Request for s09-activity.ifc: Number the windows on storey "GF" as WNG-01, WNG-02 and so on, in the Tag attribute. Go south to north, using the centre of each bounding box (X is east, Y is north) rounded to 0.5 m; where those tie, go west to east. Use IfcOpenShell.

First a look at what the model holds.

```python
import ifcopenshell
import ifcopenshell.util.element
import ifcopenshell.util.placement

model = ifcopenshell.open("s09-activity.ifc")
print(model.schema)
storey = next(s for s in model.by_type("IfcBuildingStorey") if s.Name == "GF")
windows = [e for e in ifcopenshell.util.element.get_decomposition(storey) if e.is_a("IfcWindow")]
for e in sorted(windows, key=lambda e: e.id()):
    origin = ifcopenshell.util.placement.get_local_placement(e.ObjectPlacement)[:3, 3]
    print(e.id(), e.Tag, e.Name, origin.round(2) + 0.0, sep=" | ")
```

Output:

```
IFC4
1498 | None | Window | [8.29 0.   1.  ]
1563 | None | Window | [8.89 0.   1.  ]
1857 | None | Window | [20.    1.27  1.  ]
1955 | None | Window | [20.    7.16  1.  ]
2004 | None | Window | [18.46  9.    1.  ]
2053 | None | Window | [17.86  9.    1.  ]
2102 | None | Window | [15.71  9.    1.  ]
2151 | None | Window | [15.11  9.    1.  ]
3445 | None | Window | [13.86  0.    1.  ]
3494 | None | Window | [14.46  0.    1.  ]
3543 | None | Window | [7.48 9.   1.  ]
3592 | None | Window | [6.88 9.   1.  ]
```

```python
import ifcopenshell
import ifcopenshell.geom
import ifcopenshell.util.element
import ifcopenshell.util.shape

model = ifcopenshell.open("s09-activity.ifc")
settings = ifcopenshell.geom.settings()
settings.set("use-world-coords", True)


def centre(element):
    shape = ifcopenshell.geom.create_shape(settings, element)
    return ifcopenshell.util.shape.get_bbox_centroid(shape.geometry)


storey = next(s for s in model.by_type("IfcBuildingStorey") if s.Name == "GF")
windows = [e for e in ifcopenshell.util.element.get_decomposition(storey) if e.is_a("IfcWindow")]

# Insertion points can sit at a corner or the storey origin, so sort by the geometry (in metres).
centres = {e: centre(e) for e in windows}
windows.sort(key=lambda e: (round(centres[e][1] / 0.5), centres[e][0]))

for i, e in enumerate(windows, start=1):
    number = f"WNG-{i:02d}"
    e.Tag = number
    print(e.id(), number)

model.write("s09-activity_edited.ifc")
```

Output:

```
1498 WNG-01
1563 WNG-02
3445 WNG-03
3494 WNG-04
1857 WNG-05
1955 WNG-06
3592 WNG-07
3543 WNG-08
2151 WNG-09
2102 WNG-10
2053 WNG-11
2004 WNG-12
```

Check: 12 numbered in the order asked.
